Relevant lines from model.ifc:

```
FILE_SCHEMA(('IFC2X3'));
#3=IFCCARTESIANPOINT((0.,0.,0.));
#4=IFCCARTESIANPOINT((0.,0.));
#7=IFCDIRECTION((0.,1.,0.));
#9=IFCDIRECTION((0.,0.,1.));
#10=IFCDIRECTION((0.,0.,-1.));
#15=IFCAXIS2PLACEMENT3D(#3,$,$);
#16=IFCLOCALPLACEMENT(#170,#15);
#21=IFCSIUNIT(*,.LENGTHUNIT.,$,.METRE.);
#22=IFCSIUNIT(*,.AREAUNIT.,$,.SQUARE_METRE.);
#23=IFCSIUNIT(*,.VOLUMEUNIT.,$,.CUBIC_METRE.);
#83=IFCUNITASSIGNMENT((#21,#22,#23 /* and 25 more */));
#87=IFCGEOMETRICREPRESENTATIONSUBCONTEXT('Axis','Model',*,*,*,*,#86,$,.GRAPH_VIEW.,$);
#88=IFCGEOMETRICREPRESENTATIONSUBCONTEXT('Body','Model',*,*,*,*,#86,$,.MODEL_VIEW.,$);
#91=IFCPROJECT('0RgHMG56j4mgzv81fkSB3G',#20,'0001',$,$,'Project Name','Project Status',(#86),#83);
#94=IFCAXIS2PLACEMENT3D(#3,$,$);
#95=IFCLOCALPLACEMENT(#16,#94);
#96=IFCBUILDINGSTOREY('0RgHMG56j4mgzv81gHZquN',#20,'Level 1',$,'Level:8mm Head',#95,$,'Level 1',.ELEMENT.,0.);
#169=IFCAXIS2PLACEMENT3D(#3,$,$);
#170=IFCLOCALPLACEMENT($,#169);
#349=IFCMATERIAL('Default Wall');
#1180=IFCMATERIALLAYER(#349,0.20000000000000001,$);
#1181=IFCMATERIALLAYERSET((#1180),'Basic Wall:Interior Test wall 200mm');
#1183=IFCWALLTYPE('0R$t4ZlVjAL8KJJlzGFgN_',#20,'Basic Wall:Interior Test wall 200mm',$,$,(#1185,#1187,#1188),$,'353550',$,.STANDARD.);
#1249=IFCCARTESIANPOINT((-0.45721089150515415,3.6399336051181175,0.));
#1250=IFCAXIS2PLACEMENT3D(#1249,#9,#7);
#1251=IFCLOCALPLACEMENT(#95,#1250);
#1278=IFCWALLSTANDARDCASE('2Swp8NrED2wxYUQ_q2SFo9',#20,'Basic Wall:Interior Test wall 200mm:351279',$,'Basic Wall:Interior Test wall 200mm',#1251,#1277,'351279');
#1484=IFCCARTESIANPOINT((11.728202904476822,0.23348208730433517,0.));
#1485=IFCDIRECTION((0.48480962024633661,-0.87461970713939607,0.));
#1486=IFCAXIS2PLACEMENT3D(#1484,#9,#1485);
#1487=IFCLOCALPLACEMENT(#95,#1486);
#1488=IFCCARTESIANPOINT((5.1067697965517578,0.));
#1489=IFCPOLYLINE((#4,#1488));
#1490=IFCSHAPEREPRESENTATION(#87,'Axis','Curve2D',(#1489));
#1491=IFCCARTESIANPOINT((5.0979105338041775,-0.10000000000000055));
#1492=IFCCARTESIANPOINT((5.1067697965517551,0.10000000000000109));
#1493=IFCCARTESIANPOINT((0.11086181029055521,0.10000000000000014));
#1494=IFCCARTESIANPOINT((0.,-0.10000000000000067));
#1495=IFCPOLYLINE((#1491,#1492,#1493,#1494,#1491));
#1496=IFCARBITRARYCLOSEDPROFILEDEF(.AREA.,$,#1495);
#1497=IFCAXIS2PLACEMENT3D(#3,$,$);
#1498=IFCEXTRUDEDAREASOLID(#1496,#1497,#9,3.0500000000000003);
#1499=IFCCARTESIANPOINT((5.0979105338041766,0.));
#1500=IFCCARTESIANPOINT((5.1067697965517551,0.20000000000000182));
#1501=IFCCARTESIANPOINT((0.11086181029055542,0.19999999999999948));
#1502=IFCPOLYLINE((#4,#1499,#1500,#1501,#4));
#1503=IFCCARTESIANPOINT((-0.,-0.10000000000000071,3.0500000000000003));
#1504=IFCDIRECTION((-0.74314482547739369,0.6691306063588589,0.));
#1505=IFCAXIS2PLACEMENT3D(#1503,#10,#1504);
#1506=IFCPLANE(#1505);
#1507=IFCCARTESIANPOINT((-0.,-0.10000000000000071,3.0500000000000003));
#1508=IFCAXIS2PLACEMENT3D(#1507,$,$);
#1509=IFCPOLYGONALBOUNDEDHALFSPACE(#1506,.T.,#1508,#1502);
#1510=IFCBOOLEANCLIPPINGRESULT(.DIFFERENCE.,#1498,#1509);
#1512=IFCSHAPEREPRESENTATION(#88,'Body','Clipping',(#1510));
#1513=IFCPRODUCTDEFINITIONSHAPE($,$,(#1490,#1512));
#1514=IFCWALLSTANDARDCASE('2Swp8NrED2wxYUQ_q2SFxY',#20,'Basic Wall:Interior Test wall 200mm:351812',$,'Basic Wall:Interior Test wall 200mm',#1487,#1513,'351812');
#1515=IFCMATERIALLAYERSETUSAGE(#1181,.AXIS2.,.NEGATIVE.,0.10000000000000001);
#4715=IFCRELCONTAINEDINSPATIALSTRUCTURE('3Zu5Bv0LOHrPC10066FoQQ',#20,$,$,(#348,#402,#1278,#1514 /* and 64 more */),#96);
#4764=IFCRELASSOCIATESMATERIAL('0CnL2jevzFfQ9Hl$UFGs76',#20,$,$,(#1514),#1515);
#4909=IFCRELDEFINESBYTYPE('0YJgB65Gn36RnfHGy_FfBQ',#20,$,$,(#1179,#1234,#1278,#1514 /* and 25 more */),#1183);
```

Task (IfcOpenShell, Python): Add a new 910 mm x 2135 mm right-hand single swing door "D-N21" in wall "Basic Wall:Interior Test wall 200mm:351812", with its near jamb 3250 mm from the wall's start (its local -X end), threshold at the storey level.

```python
import numpy as np
import ifcopenshell
import ifcopenshell.api.feature
import ifcopenshell.api.geometry
import ifcopenshell.api.root
import ifcopenshell.api.spatial
import ifcopenshell.api.type
import ifcopenshell.geom
import ifcopenshell.util.element
import ifcopenshell.util.placement
import ifcopenshell.util.representation
import ifcopenshell.util.shape
import ifcopenshell.util.unit

model = ifcopenshell.open("model.ifc")
unit_scale = ifcopenshell.util.unit.calculate_unit_scale(model)
settings = ifcopenshell.geom.settings()


def volume(element):
    """Net volume in cubic metres, openings subtracted."""
    shape = ifcopenshell.geom.create_shape(settings, element)
    return ifcopenshell.util.shape.get_volume(shape.geometry)


wall = model.by_guid("2Swp8NrED2wxYUQ_q2SFxY")
storey = ifcopenshell.util.element.get_container(wall, ifc_class="IfcBuildingStorey")
context = ifcopenshell.util.representation.get_context(model, "Model", "Body", "MODEL_VIEW")
before = volume(wall)

width, height, from_end, sill = 0.91, 2.135, 3.25, 0.0  # metres

# The wall runs along its own X axis, and the end named is its -X end.
wall_shape = ifcopenshell.geom.create_shape(settings, wall)
x, y, z = ifcopenshell.util.shape.get_vertices(wall_shape.geometry).T
start = x.min() + from_end
face, thickness = float(y.min()), float(y.max() - y.min())
wall_matrix = ifcopenshell.util.placement.get_local_placement(wall.ObjectPlacement)
level = ifcopenshell.util.placement.get_local_placement(storey.ObjectPlacement)[2, 3]


def in_wall(x, y):
    """Placement at x, y metres in the wall's axes, at sill height."""
    matrix = wall_matrix.copy()
    matrix[:, 3] = wall_matrix @ np.array([x / unit_scale, y / unit_scale, 0.0, 1.0])
    matrix[2, 3] = level + sill / unit_scale
    return matrix


# Opening: a box that overshoots both wall faces by 50 mm.
opening = ifcopenshell.api.root.create_entity(model, ifc_class="IfcOpeningElement")
box = ifcopenshell.api.geometry.add_wall_representation(
    model, context=context, length=width, height=height, thickness=thickness + 0.1
)
ifcopenshell.api.geometry.assign_representation(model, product=opening, representation=box)
ifcopenshell.api.geometry.edit_object_placement(model, product=opening, matrix=in_wall(start, face - 0.05), is_si=False)
ifcopenshell.api.feature.add_feature(model, feature=opening, element=wall)

door = ifcopenshell.api.root.create_entity(model, ifc_class="IfcDoor", name="D-N21")
door.OverallWidth, door.OverallHeight = width / unit_scale, height / unit_scale
body = ifcopenshell.api.geometry.add_door_representation(
    model,
    context=context,
    overall_width=door.OverallWidth,
    overall_height=door.OverallHeight,
    operation_type="SINGLE_SWING_RIGHT",
    lining_properties={"LiningDepth": thickness / unit_scale, "ThresholdDepth": thickness / unit_scale},
)
ifcopenshell.api.geometry.assign_representation(model, product=door, representation=body)
ifcopenshell.api.spatial.assign_container(model, products=[door], relating_structure=storey)
fills = ifcopenshell.api.feature.add_filling(model, opening=opening, element=door)
fills.OwnerHistory = door.OwnerHistory  # required in IFC2X3

# IFC2X3 keeps the operation on the door style.
style = ifcopenshell.api.root.create_entity(model, ifc_class="IfcDoorStyle", name="D-N21")
style.OperationType, style.ConstructionType = "SINGLE_SWING_RIGHT", "NOTDEFINED"
style.ParameterTakesPrecedence = style.Sizeable = False
ifcopenshell.api.type.assign_type(model, related_objects=[door], relating_type=style)

# The lining spans the wall, so the door starts at the wall face.
ifcopenshell.api.geometry.edit_object_placement(model, product=door, matrix=in_wall(start, face), is_si=False)

after = volume(wall)

print(f"wall volume {before:.3f} -> {after:.3f} m3")

model.write("model_rev.ifc")
```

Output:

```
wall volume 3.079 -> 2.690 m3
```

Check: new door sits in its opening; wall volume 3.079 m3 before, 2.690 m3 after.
